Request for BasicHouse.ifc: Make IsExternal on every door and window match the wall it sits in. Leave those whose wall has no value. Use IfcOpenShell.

First a look at what the model holds.

```python
import ifcopenshell
import ifcopenshell.util.element

model = ifcopenshell.open("BasicHouse.ifc")
print(model.schema)
seen = {}
for e in model.by_type("IfcDoor") + model.by_type("IfcWindow"):
    if not e.FillsVoids:
        continue
    host = e.FillsVoids[0].RelatingOpeningElement.VoidsElements[0].RelatingBuildingElement
    own = ifcopenshell.util.element.get_pset(e, f"Pset_{e.is_a()[3:].removesuffix('StandardCase')}Common", "IsExternal")
    wall = ifcopenshell.util.element.get_pset(host, "Pset_WallCommon", "IsExternal")
    seen[e.is_a(), own, wall] = seen.get((e.is_a(), own, wall), 0) + 1
for (cls, own, wall), count in sorted(seen.items(), key=str):
    print(count, cls, "IsExternal:", own, "| host wall:", wall)
```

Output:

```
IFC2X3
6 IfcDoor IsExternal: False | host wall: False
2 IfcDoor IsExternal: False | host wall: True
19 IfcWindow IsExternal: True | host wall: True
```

```python
import ifcopenshell
import ifcopenshell.api.pset
import ifcopenshell.util.element

model = ifcopenshell.open("BasicHouse.ifc")

count = 0
for ifc_class, pset_name in (("IfcDoor", "Pset_DoorCommon"), ("IfcWindow", "Pset_WindowCommon")):
    for e in model.by_type(ifc_class):
        if not e.FillsVoids:
            continue
        host = e.FillsVoids[0].RelatingOpeningElement.VoidsElements[0].RelatingBuildingElement
        external = ifcopenshell.util.element.get_pset(host, "Pset_WallCommon", "IsExternal")
        if external is None or ifcopenshell.util.element.get_pset(e, pset_name, "IsExternal") == external:
            continue
        pset = ifcopenshell.api.pset.add_pset(model, product=e, name=pset_name)
        ifcopenshell.api.pset.edit_pset(model, pset=pset, properties={"IsExternal": external})
        count += 1

print(count, "updated")

model.write("BasicHouse_updated.ifc")
```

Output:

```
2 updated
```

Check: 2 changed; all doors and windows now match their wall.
